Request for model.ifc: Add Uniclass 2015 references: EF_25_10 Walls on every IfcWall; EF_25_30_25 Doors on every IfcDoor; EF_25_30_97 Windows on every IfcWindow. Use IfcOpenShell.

First a look at what the model holds.

```python
import ifcopenshell

model = ifcopenshell.open("model.ifc")
print(model.schema)
print("classifications:", [c.Name for c in model.by_type("IfcClassification")])
for ifc_class in ("IfcDoor", "IfcRoof", "IfcStair", "IfcWall", "IfcWindow"):
    print(ifc_class, len(model.by_type(ifc_class)))
```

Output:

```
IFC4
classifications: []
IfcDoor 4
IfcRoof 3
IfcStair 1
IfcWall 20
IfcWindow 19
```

```python
import ifcopenshell
import ifcopenshell.api.classification

model = ifcopenshell.open("model.ifc")

system = ifcopenshell.api.classification.add_classification(model, classification="Uniclass 2015")

codes = {
    "IfcWall": ("EF_25_10", "Walls"),
    "IfcDoor": ("EF_25_30_25", "Doors"),
    "IfcWindow": ("EF_25_30_97", "Windows"),
}
for ifc_class, (code, name) in codes.items():
    products = model.by_type(ifc_class)
    ifcopenshell.api.classification.add_reference(
        model, products=products, classification=system, identification=code, name=name
    )
    print(code, len(products))

model.write("model_rev.ifc")
```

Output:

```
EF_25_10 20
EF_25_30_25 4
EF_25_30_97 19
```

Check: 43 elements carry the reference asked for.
